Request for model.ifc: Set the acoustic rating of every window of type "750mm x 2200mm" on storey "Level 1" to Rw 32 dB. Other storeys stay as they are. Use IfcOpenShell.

First a look at what the model holds.

```python
import ifcopenshell
import ifcopenshell.util.element

model = ifcopenshell.open("model.ifc")
print(model.schema)
storey = next(s for s in model.by_type("IfcBuildingStorey") if s.Name == "Level 1")
windows = [e for e in ifcopenshell.util.element.get_decomposition(storey) if e.is_a("IfcWindow")]
seen = {}
for e in windows:
    element_type = ifcopenshell.util.element.get_type(e)
    key = (element_type.Name if element_type != e and element_type else None, ifcopenshell.util.element.get_pset(e, "Pset_WindowCommon", "AcousticRating"))
    seen[key] = seen.get(key, 0) + 1
for (name, value), count in sorted(seen.items(), key=str):
    print(count, "x", name, "|", value)
```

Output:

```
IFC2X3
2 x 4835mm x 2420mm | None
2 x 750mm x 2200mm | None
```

```python
import ifcopenshell
import ifcopenshell.api.pset
import ifcopenshell.util.element

model = ifcopenshell.open("model.ifc")

storey = next(s for s in model.by_type("IfcBuildingStorey") if s.Name == "Level 1")
windows = [e for e in ifcopenshell.util.element.get_decomposition(storey) if e.is_a("IfcWindow")]

count = 0
for e in windows:
    element_type = ifcopenshell.util.element.get_type(e)
    if element_type in (None, e) or element_type.Name != "750mm x 2200mm":
        continue
    # add_pset returns the element's existing set when there is one.
    pset = ifcopenshell.api.pset.add_pset(model, product=e, name="Pset_WindowCommon")
    ifcopenshell.api.pset.edit_pset(model, pset=pset, properties={"AcousticRating": "Rw 32 dB"})
    count += 1

print(count, "windows updated")

model.write("model_rev.ifc")
```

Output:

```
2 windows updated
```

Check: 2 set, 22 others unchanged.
